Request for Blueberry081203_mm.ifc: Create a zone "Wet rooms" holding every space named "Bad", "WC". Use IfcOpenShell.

First a look at what the model holds.

```python
import ifcopenshell

model = ifcopenshell.open("Blueberry081203_mm.ifc")
print(model.schema)
seen = {}
for space in model.by_type("IfcSpace"):
    seen[space.LongName] = seen.get(space.LongName, 0) + 1
for name, count in sorted(seen.items(), key=str):
    print(count, "x", name)
print("zones:", [z.Name for z in model.by_type("IfcZone")][:20])
```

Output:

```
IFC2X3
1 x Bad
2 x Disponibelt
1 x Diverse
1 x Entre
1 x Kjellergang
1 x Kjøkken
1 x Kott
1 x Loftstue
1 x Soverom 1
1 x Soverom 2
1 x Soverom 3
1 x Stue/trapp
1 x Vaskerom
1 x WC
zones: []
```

```python
import ifcopenshell
import ifcopenshell.api.group
import ifcopenshell.api.root

model = ifcopenshell.open("Blueberry081203_mm.ifc")

names = {"Bad", "WC"}
spaces = [s for s in model.by_type("IfcSpace") if s.LongName in names]

zone = ifcopenshell.api.root.create_entity(model, ifc_class="IfcZone", name="Wet rooms")
ifcopenshell.api.group.assign_group(model, products=spaces, group=zone)
print(len(spaces), "spaces in", zone.Name)

model.write("Blueberry081203_mm_edited.ifc")
```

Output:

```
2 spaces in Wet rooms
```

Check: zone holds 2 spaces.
